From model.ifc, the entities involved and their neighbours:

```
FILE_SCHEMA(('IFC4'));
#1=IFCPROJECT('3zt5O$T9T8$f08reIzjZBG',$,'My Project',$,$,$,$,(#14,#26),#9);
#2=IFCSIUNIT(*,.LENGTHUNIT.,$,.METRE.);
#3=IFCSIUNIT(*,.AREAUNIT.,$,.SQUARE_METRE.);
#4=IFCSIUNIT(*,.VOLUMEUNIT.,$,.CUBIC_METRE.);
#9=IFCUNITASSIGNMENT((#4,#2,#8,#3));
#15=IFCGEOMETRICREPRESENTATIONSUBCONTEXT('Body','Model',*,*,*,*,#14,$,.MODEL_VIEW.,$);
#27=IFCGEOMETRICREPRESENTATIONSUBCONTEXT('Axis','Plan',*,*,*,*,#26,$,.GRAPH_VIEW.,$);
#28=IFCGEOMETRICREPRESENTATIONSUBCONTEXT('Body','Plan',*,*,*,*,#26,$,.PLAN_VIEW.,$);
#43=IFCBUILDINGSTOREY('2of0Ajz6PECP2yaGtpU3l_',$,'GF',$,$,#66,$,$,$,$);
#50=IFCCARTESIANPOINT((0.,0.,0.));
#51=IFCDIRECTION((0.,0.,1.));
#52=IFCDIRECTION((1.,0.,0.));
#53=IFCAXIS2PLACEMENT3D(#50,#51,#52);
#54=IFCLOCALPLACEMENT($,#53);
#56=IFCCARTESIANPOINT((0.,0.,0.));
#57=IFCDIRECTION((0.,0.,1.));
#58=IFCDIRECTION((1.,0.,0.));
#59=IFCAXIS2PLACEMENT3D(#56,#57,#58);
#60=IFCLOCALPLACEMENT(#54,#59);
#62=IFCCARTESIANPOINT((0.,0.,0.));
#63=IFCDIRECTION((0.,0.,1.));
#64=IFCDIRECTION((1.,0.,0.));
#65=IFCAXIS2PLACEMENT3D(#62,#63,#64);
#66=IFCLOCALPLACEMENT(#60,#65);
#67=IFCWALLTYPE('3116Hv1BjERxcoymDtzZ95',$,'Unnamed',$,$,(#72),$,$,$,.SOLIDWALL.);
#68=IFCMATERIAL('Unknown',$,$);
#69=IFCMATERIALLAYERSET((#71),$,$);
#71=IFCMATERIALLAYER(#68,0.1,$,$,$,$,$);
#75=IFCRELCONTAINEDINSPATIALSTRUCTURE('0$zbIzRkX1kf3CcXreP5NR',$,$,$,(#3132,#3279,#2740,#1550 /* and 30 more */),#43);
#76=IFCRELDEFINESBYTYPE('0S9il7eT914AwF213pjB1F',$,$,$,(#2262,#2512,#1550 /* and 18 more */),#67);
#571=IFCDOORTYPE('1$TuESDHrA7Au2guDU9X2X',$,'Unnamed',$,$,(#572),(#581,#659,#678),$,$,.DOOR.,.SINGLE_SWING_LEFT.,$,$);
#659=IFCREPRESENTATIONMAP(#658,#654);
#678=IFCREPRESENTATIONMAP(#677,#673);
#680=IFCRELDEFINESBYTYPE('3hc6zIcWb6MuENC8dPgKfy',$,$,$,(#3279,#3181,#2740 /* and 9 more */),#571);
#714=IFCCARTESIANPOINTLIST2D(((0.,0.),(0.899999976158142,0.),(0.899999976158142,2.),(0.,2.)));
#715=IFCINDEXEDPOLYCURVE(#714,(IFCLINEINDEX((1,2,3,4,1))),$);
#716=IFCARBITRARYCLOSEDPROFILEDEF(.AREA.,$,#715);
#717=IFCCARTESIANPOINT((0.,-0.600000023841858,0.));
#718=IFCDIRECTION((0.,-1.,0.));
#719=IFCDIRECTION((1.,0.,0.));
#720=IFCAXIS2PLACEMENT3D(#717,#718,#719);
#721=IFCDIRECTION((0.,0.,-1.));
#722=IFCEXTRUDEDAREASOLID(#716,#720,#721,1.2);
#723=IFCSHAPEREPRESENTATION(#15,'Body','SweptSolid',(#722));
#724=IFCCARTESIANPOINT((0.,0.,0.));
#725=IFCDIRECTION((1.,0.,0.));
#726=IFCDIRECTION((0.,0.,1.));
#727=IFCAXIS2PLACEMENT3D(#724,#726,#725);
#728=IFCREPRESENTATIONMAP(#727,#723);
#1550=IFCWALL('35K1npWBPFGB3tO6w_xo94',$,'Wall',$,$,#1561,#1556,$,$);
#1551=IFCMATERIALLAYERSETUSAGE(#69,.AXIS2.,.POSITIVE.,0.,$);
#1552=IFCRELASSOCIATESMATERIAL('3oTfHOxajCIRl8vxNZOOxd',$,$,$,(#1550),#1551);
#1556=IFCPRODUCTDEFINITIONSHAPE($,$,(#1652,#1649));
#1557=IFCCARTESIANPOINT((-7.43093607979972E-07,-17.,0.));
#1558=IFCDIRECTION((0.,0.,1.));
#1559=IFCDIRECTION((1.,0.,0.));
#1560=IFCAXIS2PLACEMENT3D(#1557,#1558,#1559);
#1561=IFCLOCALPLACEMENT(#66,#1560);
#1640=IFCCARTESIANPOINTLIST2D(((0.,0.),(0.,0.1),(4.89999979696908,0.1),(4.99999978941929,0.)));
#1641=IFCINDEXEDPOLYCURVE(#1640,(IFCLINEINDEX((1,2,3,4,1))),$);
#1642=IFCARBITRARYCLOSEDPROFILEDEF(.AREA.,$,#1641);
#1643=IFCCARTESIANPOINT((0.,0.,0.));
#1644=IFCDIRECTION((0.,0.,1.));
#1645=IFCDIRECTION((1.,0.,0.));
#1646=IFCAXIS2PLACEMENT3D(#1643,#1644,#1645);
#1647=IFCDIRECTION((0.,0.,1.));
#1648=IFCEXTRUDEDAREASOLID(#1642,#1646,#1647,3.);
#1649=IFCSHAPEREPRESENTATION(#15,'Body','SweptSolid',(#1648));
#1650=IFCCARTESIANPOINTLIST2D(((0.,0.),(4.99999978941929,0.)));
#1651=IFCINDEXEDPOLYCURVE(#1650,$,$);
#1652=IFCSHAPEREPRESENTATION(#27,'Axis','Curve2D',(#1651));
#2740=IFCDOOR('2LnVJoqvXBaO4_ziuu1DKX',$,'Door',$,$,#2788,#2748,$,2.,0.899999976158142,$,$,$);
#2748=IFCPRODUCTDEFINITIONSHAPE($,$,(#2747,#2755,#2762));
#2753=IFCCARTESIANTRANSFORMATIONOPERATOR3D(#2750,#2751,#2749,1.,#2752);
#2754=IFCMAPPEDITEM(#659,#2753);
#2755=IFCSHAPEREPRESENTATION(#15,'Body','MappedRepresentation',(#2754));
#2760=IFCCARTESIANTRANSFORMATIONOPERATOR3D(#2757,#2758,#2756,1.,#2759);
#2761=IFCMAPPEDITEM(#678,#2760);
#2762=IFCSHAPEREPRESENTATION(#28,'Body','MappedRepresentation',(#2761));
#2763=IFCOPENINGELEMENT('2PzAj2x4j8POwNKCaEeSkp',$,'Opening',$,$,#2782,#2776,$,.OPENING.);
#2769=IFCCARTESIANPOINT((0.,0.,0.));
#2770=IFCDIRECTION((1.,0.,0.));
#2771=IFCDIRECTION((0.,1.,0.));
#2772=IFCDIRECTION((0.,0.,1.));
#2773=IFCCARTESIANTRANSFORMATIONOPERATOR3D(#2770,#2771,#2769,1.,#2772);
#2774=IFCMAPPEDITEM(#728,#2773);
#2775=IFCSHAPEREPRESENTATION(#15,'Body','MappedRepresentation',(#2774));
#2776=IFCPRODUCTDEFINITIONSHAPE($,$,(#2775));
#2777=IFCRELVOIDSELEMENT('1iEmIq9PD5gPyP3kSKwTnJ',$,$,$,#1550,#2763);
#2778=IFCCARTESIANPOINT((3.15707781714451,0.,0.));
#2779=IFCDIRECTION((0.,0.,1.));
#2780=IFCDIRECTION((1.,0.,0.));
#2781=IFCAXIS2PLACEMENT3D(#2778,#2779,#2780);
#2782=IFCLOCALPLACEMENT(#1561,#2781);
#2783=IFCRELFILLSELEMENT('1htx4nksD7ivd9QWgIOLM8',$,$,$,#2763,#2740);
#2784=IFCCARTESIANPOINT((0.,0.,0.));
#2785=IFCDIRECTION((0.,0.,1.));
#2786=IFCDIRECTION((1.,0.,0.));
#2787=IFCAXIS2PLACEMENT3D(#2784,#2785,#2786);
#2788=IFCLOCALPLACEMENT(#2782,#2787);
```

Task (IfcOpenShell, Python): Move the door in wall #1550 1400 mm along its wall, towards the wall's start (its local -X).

```python
import ifcopenshell
import ifcopenshell.api.geometry
import ifcopenshell.util.placement
import ifcopenshell.util.unit

model = ifcopenshell.open("model.ifc")
unit_scale = ifcopenshell.util.unit.calculate_unit_scale(model)

door = model.by_guid("2LnVJoqvXBaO4_ziuu1DKX")
opening = door.FillsVoids[0].RelatingOpeningElement
wall = opening.VoidsElements[0].RelatingBuildingElement

wall_matrix = ifcopenshell.util.placement.get_local_placement(wall.ObjectPlacement)
shift = wall_matrix[:3, 0] * -1.4 / unit_scale
before = ifcopenshell.util.placement.get_local_placement(door.ObjectPlacement)[:3, 3].copy()

# The door is placed relative to its opening, so it follows when the opening moves.
matrix = ifcopenshell.util.placement.get_local_placement(opening.ObjectPlacement)
matrix[:3, 3] += shift
ifcopenshell.api.geometry.edit_object_placement(
    model, product=opening, matrix=matrix, is_si=False, should_transform_children=True
)

after = ifcopenshell.util.placement.get_local_placement(door.ObjectPlacement)[:3, 3]
print("door moved by", (after - before).round(3) + 0.0)

model.write("model_v2.ifc")
```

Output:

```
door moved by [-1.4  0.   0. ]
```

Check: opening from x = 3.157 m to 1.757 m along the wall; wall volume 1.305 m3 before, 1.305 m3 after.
